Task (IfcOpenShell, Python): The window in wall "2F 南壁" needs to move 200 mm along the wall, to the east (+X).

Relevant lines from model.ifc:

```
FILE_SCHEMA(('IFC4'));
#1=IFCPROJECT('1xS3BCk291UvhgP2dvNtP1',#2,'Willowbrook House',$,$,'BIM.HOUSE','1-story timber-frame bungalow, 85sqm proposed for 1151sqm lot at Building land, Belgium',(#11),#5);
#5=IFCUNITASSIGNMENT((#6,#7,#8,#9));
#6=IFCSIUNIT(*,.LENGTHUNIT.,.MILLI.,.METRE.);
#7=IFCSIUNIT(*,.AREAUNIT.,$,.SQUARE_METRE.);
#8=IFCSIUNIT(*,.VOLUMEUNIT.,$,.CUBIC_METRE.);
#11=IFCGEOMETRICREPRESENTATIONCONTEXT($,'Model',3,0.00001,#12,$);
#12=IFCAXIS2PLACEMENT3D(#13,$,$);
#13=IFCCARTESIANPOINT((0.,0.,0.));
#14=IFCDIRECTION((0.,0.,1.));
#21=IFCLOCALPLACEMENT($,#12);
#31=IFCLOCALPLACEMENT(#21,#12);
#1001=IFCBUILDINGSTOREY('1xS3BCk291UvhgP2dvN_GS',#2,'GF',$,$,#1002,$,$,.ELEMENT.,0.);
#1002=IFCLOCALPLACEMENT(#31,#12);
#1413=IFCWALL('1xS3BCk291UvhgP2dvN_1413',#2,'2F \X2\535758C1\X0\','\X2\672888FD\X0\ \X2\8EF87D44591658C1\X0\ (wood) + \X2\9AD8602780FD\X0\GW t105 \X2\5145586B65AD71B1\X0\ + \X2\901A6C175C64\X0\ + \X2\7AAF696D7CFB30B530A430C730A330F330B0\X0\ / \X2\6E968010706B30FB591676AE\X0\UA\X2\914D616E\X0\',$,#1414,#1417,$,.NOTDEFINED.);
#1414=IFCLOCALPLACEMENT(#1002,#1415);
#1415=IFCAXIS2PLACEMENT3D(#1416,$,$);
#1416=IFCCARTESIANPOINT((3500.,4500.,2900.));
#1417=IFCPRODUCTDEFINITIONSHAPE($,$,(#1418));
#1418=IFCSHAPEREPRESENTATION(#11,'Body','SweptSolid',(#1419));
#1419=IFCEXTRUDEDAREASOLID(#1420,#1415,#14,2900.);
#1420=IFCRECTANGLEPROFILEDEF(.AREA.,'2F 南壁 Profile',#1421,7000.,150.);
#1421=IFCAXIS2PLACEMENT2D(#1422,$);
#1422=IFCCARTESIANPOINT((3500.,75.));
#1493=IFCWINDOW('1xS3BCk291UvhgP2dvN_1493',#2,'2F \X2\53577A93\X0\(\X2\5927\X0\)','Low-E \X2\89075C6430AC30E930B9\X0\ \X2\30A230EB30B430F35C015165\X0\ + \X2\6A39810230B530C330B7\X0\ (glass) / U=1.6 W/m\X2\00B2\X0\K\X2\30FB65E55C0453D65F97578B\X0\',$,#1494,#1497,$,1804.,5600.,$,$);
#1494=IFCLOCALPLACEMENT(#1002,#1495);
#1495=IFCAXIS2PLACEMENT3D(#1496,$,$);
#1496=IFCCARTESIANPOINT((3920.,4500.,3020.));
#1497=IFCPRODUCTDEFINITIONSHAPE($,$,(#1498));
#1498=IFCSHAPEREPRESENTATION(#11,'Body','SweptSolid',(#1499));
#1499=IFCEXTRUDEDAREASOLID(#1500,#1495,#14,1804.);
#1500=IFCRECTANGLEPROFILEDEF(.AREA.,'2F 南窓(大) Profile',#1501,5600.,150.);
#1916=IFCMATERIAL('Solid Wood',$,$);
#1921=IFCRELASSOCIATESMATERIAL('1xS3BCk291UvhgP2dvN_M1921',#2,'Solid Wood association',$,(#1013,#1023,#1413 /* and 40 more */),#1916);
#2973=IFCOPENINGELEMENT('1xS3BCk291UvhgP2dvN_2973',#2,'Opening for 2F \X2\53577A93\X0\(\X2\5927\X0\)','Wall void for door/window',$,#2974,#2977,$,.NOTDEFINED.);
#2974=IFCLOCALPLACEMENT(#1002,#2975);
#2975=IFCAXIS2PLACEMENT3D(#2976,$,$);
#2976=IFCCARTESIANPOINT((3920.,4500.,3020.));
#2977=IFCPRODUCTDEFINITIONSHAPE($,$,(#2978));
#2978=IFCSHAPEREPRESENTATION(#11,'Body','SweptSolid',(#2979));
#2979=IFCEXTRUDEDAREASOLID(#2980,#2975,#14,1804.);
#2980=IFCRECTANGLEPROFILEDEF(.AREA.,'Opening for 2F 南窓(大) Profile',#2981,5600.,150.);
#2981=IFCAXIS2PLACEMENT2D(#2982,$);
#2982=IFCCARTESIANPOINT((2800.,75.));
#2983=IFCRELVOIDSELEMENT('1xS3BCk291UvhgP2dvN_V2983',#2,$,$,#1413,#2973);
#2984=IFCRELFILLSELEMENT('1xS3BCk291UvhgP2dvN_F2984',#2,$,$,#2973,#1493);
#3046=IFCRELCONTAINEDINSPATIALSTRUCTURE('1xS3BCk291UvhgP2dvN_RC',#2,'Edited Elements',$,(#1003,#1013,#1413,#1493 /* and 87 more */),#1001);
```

```python
import ifcopenshell
import ifcopenshell.api.geometry
import ifcopenshell.util.placement
import ifcopenshell.util.unit

model = ifcopenshell.open("model.ifc")
unit_scale = ifcopenshell.util.unit.calculate_unit_scale(model)

window = model.by_id(1493)
opening = window.FillsVoids[0].RelatingOpeningElement
wall = opening.VoidsElements[0].RelatingBuildingElement

wall_matrix = ifcopenshell.util.placement.get_local_placement(wall.ObjectPlacement)
shift = wall_matrix[:3, 0] * 0.2 / unit_scale
before = ifcopenshell.util.placement.get_local_placement(window.ObjectPlacement)[:3, 3].copy()

# The window is not placed relative to its opening, so move both.
for product in (opening, window):
    matrix = ifcopenshell.util.placement.get_local_placement(product.ObjectPlacement)
    matrix[:3, 3] += shift
    ifcopenshell.api.geometry.edit_object_placement(model, product=product, matrix=matrix, is_si=False)

after = ifcopenshell.util.placement.get_local_placement(window.ObjectPlacement)[:3, 3]
print("window moved by", (after - before).round(3) + 0.0)

model.write("model_edited.ifc")
```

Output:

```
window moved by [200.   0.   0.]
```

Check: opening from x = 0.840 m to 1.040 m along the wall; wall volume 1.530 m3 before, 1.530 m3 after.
